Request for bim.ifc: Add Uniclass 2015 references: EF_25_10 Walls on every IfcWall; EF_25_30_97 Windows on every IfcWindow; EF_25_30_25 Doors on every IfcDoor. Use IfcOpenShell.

First a look at what the model holds.

```python
import ifcopenshell

model = ifcopenshell.open("bim.ifc")
print(model.schema)
print("classifications:", [c.Name for c in model.by_type("IfcClassification")])
for ifc_class in ("IfcDoor", "IfcRoof", "IfcStair", "IfcWall", "IfcWindow"):
    print(ifc_class, len(model.by_type(ifc_class)))
```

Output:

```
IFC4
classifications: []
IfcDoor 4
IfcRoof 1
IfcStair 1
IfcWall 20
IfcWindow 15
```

```python
import ifcopenshell
import ifcopenshell.api.classification

model = ifcopenshell.open("bim.ifc")

system = ifcopenshell.api.classification.add_classification(model, classification="Uniclass 2015")

codes = {
    "IfcWall": ("EF_25_10", "Walls"),
    "IfcWindow": ("EF_25_30_97", "Windows"),
    "IfcDoor": ("EF_25_30_25", "Doors"),
}
for ifc_class, (code, name) in codes.items():
    products = model.by_type(ifc_class)
    ifcopenshell.api.classification.add_reference(
        model, products=products, classification=system, identification=code, name=name
    )
    print(code, len(products))

model.write("bim-out.ifc")
```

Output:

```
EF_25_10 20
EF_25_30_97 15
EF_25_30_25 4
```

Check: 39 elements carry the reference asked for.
